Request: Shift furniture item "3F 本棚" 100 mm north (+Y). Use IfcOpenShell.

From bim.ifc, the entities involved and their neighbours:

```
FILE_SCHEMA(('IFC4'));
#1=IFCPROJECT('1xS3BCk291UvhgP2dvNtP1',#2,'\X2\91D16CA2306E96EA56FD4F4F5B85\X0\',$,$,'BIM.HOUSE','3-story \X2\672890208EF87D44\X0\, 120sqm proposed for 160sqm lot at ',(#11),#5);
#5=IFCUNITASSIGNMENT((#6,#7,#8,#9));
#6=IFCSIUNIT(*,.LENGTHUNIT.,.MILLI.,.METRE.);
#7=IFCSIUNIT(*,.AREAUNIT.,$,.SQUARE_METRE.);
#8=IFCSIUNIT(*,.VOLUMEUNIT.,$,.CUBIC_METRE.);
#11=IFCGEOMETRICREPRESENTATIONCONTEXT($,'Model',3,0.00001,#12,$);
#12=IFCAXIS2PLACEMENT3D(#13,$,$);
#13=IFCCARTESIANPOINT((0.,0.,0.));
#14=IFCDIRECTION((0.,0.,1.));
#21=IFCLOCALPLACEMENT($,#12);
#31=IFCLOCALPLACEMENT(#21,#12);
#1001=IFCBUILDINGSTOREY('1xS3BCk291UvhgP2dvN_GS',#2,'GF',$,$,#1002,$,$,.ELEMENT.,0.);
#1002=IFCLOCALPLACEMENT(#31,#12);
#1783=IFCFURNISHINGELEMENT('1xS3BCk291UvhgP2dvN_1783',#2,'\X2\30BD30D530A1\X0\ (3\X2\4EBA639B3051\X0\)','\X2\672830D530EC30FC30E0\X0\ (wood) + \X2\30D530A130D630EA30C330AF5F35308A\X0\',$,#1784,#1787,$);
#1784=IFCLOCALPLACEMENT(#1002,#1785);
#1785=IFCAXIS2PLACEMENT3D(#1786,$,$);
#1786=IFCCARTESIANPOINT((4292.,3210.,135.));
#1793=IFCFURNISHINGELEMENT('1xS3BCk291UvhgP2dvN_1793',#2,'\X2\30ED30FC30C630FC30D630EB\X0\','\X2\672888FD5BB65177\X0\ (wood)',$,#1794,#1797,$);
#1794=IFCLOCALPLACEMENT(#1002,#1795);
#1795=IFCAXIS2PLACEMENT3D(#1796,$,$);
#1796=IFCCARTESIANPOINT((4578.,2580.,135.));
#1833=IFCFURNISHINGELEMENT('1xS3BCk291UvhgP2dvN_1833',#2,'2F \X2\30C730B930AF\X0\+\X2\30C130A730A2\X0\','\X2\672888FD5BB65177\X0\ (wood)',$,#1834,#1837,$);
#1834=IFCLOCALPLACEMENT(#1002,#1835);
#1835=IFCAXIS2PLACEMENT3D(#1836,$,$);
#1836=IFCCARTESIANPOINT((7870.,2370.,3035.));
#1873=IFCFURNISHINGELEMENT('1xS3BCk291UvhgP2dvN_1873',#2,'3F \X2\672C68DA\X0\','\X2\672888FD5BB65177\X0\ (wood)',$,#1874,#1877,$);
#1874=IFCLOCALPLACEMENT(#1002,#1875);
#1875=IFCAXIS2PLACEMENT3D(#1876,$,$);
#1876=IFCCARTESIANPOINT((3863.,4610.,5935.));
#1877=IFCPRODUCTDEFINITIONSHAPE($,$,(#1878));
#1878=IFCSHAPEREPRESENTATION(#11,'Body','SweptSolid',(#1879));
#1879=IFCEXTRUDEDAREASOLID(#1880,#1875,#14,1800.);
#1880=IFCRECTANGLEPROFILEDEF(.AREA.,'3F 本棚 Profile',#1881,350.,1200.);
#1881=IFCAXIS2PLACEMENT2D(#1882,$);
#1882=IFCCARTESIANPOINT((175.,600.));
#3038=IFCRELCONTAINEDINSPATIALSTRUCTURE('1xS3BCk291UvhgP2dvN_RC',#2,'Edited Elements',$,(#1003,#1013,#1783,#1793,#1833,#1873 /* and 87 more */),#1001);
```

```python
import ifcopenshell
import ifcopenshell.api.geometry
import ifcopenshell.util.placement
import ifcopenshell.util.unit

model = ifcopenshell.open("bim.ifc")
unit_scale = ifcopenshell.util.unit.calculate_unit_scale(model)

item = model.by_guid("1xS3BCk291UvhgP2dvN_1873")
matrix = ifcopenshell.util.placement.get_local_placement(item.ObjectPlacement)
matrix[1, 3] += 0.1 / unit_scale
ifcopenshell.api.geometry.edit_object_placement(model, product=item, matrix=matrix, is_si=False)

print(ifcopenshell.util.placement.get_local_placement(item.ObjectPlacement).round(3) + 0.0)

model.write("bim_v2.ifc")
```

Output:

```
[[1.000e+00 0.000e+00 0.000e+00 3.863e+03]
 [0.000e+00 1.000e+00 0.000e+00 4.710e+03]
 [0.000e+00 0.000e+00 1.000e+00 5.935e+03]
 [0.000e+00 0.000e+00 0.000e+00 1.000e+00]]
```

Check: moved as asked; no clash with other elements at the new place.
